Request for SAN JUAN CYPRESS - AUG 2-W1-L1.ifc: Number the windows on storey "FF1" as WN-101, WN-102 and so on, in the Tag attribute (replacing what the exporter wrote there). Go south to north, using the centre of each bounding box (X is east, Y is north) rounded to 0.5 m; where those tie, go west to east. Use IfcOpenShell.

First a look at what the model holds.

```python
import ifcopenshell
import ifcopenshell.util.element
import ifcopenshell.util.placement

model = ifcopenshell.open("SAN JUAN CYPRESS - AUG 2-W1-L1.ifc")
print(model.schema)
storey = next(s for s in model.by_type("IfcBuildingStorey") if s.Name == "FF1")
windows = [e for e in ifcopenshell.util.element.get_decomposition(storey) if e.is_a("IfcWindow")]
for e in sorted(windows, key=lambda e: e.id()):
    origin = ifcopenshell.util.placement.get_local_placement(e.ObjectPlacement)[:3, 3]
    print(e.id(), e.Tag, e.Name, origin.round(2) + 0.0, sep=" | ")
```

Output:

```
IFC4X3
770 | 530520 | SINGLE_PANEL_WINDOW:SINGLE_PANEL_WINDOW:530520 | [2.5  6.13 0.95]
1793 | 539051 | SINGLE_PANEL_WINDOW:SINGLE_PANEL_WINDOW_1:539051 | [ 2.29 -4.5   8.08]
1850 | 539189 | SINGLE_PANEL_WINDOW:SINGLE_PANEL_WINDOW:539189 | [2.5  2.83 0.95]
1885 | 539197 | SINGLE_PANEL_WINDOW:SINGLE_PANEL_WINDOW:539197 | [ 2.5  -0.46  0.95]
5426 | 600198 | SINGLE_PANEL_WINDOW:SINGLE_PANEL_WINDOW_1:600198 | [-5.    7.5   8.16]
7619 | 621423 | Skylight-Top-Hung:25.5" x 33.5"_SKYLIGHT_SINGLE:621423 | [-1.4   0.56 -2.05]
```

```python
import ifcopenshell
import ifcopenshell.geom
import ifcopenshell.util.element
import ifcopenshell.util.shape

model = ifcopenshell.open("SAN JUAN CYPRESS - AUG 2-W1-L1.ifc")
settings = ifcopenshell.geom.settings()
settings.set("use-world-coords", True)


def centre(element):
    shape = ifcopenshell.geom.create_shape(settings, element)
    return ifcopenshell.util.shape.get_bbox_centroid(shape.geometry)


storey = next(s for s in model.by_type("IfcBuildingStorey") if s.Name == "FF1")
windows = [e for e in ifcopenshell.util.element.get_decomposition(storey) if e.is_a("IfcWindow")]

# Insertion points can sit at a corner or the storey origin, so sort by the geometry (in metres).
centres = {e: centre(e) for e in windows}
windows.sort(key=lambda e: (round(centres[e][1] / 0.5), centres[e][0]))

for i, e in enumerate(windows, start=1):
    number = f"WN-1{i:02d}"
    e.Tag = number
    print(e.id(), number)

model.write("SAN JUAN CYPRESS - AUG 2-W1-L1_rev.ifc")
```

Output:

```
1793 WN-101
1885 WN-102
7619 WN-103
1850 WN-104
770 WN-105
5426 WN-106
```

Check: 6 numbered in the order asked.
